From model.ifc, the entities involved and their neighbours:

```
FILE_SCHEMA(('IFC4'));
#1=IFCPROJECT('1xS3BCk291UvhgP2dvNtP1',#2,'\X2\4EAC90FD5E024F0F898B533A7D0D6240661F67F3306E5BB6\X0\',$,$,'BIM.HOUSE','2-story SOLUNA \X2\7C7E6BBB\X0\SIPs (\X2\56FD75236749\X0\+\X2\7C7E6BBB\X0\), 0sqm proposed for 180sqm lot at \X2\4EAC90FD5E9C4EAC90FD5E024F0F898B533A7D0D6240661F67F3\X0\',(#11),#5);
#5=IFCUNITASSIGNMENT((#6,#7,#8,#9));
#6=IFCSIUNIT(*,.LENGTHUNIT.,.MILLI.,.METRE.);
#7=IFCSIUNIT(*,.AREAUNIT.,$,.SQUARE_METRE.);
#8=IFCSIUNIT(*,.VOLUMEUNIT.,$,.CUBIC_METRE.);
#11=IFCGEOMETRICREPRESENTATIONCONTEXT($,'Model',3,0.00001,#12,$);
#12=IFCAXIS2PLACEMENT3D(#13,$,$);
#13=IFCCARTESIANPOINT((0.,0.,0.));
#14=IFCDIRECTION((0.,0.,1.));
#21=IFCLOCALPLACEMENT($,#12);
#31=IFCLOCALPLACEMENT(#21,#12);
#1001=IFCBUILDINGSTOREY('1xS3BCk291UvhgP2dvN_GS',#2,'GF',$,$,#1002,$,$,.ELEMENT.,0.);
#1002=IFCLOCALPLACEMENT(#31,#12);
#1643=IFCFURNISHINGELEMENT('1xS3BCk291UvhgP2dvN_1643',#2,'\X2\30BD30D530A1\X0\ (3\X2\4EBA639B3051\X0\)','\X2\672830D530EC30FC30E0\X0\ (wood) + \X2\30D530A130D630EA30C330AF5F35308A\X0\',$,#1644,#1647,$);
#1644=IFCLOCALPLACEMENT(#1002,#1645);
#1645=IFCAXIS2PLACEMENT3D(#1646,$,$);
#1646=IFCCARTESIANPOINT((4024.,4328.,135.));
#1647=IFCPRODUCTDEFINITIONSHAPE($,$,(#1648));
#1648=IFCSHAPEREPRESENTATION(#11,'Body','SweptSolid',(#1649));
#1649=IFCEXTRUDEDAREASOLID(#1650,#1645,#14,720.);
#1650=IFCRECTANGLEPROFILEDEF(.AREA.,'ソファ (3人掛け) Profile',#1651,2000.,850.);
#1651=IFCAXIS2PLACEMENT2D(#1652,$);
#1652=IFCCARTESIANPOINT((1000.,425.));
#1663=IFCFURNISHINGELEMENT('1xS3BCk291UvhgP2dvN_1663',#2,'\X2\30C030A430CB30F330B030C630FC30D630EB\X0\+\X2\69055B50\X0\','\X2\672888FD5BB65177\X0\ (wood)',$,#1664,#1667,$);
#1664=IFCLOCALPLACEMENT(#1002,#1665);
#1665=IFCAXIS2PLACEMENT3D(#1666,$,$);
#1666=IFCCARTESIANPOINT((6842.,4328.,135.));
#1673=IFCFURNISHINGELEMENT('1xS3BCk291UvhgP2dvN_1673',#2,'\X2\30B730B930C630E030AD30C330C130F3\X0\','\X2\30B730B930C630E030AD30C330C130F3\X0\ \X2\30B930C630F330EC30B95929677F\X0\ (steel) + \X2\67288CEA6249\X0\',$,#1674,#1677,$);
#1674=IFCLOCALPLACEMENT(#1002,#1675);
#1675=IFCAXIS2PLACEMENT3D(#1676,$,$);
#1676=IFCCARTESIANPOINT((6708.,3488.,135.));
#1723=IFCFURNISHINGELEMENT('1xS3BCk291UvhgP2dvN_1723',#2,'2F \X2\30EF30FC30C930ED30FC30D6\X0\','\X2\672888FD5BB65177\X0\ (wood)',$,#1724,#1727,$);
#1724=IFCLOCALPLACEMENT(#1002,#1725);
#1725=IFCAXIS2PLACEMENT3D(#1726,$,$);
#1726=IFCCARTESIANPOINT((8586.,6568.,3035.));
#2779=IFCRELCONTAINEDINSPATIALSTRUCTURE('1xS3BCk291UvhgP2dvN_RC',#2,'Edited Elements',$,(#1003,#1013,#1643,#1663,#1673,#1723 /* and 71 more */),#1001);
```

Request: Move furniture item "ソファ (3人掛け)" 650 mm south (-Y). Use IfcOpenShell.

```python
import ifcopenshell
import ifcopenshell.api.geometry
import ifcopenshell.util.placement

model = ifcopenshell.open("model.ifc")

item = model.by_guid("1xS3BCk291UvhgP2dvN_1643")
matrix = ifcopenshell.util.placement.get_local_placement(item.ObjectPlacement)
matrix[1, 3] -= 650.0
ifcopenshell.api.geometry.edit_object_placement(model, product=item, matrix=matrix, is_si=False)

print(ifcopenshell.util.placement.get_local_placement(item.ObjectPlacement).round(3) + 0.0)

model.write("model_updated.ifc")
```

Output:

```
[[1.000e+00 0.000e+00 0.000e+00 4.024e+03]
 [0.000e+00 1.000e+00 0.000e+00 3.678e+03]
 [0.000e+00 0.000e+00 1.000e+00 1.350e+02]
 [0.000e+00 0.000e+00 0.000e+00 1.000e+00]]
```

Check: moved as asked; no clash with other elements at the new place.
